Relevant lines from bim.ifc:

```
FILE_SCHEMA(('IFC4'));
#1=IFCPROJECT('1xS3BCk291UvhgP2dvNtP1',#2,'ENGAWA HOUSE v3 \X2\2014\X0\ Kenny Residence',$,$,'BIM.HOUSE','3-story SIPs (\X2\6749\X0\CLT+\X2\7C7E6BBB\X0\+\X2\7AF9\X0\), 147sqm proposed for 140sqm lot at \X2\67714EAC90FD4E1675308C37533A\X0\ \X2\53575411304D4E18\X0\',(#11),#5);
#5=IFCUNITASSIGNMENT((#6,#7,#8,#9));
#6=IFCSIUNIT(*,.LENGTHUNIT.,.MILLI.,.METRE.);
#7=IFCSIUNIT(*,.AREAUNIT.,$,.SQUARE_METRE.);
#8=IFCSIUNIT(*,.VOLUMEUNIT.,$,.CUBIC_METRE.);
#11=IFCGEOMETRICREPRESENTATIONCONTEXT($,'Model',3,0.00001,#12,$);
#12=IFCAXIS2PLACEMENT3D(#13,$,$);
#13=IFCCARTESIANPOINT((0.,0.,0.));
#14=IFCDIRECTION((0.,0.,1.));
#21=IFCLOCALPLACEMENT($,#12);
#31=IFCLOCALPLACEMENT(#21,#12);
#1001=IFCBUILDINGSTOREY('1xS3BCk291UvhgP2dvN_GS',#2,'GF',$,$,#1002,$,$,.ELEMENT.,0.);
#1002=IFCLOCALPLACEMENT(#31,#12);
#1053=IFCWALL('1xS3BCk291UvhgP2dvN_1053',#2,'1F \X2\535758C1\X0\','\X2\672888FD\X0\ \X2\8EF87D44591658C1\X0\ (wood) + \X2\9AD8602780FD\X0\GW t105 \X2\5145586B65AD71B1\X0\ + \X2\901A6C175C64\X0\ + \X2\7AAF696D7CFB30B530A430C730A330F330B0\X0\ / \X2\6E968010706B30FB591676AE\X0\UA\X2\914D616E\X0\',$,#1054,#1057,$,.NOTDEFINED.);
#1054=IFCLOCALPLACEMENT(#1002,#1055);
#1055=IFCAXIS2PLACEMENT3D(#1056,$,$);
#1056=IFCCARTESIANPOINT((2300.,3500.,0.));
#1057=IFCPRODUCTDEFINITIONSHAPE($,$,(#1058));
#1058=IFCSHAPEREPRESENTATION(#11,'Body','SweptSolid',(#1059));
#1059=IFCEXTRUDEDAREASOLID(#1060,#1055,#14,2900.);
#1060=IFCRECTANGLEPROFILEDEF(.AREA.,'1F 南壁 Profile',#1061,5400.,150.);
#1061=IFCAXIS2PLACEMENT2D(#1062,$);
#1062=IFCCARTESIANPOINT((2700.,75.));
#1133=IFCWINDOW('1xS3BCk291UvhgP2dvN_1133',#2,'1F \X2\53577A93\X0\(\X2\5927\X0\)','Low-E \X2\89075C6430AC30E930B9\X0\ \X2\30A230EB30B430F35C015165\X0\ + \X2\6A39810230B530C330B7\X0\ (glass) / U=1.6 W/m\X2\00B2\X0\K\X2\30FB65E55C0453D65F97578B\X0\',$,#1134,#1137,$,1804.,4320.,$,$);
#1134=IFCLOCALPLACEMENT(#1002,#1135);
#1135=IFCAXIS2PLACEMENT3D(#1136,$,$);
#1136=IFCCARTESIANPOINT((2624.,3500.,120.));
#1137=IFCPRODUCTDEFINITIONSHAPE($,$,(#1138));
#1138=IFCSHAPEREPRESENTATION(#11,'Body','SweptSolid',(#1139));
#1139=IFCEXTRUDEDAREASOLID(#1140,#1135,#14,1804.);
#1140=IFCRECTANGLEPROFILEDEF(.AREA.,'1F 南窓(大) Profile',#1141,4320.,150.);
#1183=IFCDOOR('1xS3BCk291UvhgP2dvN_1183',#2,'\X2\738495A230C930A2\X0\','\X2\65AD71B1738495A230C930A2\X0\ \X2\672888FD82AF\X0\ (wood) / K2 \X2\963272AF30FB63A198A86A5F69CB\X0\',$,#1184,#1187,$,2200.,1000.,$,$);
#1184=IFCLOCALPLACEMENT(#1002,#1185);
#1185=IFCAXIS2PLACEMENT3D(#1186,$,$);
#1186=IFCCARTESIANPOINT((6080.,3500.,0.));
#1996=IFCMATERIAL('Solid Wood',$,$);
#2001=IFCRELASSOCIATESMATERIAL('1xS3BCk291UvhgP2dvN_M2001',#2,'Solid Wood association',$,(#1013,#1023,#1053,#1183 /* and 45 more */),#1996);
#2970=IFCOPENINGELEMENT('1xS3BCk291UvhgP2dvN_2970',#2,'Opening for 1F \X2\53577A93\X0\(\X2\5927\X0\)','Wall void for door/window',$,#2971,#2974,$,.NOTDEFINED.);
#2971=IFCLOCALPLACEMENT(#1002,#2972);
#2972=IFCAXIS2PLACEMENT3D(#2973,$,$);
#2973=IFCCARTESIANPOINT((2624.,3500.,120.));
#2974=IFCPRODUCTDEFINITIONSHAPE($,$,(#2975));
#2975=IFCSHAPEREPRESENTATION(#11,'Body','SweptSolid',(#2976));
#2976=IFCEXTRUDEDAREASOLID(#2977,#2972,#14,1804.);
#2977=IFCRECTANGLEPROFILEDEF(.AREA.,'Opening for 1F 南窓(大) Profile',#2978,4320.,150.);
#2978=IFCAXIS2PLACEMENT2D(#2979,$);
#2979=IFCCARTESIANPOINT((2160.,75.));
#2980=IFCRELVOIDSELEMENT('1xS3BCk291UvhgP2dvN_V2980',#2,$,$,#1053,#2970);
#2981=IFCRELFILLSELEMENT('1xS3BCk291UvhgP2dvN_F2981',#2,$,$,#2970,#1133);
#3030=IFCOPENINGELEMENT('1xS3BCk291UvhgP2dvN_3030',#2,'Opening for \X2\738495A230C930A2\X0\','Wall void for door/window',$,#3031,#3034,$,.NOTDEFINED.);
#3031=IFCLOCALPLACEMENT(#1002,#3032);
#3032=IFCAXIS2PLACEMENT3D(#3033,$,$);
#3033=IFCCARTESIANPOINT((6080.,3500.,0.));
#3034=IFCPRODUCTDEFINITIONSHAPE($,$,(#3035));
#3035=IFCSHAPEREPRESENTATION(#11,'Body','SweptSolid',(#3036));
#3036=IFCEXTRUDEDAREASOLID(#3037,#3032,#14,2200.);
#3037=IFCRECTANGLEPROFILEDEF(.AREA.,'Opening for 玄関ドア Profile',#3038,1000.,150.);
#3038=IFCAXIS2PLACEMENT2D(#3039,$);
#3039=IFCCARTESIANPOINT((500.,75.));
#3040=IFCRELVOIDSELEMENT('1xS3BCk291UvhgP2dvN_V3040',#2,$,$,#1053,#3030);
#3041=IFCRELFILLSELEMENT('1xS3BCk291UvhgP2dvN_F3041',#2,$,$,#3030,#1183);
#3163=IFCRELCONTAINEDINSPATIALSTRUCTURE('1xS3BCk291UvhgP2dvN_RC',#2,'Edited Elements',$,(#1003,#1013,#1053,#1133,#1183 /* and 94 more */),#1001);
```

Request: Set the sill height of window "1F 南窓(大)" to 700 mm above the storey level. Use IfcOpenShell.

```python
import numpy as np
import ifcopenshell
import ifcopenshell.api.geometry
import ifcopenshell.geom
import ifcopenshell.util.element
import ifcopenshell.util.placement
import ifcopenshell.util.shape
import ifcopenshell.util.unit

model = ifcopenshell.open("bim.ifc")
unit_scale = ifcopenshell.util.unit.calculate_unit_scale(model)

window = model.by_guid("1xS3BCk291UvhgP2dvN_1133")
opening = window.FillsVoids[0].RelatingOpeningElement
storey = ifcopenshell.util.element.get_container(window, ifc_class="IfcBuildingStorey")
level = ifcopenshell.util.placement.get_local_placement(storey.ObjectPlacement)[2, 3]

# The opening's origin need not be at the sill, so measure its lowest point.
shape = ifcopenshell.geom.create_shape(ifcopenshell.geom.settings(), opening)
bottom = ifcopenshell.util.shape.get_shape_bottom_elevation(shape, shape.geometry) / unit_scale
dz = level + 700.0 - bottom

shift = np.array([0.0, 0.0, dz])
# The window is not placed relative to its opening, so move both.
for product in (opening, window):
    matrix = ifcopenshell.util.placement.get_local_placement(product.ObjectPlacement)
    matrix[:3, 3] += shift
    ifcopenshell.api.geometry.edit_object_placement(model, product=product, matrix=matrix, is_si=False)

print(f"moved by {dz * unit_scale:+.3f} m")

model.write("bim_rev.ifc")
```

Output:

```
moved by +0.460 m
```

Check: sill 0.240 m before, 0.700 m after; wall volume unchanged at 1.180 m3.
